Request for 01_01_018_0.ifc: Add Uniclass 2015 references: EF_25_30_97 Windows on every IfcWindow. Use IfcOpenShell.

First a look at what the model holds.

```python
import ifcopenshell

model = ifcopenshell.open("01_01_018_0.ifc")
print(model.schema)
print("classifications:", [c.Name for c in model.by_type("IfcClassification")])
for ifc_class in ("IfcDoor", "IfcRoof", "IfcStair", "IfcWall", "IfcWindow"):
    print(ifc_class, len(model.by_type(ifc_class)))
```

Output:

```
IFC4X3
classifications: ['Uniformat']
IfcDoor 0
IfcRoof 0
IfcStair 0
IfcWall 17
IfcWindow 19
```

```python
import ifcopenshell
import ifcopenshell.api.classification

model = ifcopenshell.open("01_01_018_0.ifc")

system = ifcopenshell.api.classification.add_classification(model, classification="Uniclass 2015")

codes = {
    "IfcWindow": ("EF_25_30_97", "Windows"),
}
for ifc_class, (code, name) in codes.items():
    products = model.by_type(ifc_class)
    ifcopenshell.api.classification.add_reference(
        model, products=products, classification=system, identification=code, name=name
    )
    print(code, len(products))

model.write("01_01_018_0_edited.ifc")
```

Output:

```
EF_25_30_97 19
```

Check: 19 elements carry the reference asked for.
